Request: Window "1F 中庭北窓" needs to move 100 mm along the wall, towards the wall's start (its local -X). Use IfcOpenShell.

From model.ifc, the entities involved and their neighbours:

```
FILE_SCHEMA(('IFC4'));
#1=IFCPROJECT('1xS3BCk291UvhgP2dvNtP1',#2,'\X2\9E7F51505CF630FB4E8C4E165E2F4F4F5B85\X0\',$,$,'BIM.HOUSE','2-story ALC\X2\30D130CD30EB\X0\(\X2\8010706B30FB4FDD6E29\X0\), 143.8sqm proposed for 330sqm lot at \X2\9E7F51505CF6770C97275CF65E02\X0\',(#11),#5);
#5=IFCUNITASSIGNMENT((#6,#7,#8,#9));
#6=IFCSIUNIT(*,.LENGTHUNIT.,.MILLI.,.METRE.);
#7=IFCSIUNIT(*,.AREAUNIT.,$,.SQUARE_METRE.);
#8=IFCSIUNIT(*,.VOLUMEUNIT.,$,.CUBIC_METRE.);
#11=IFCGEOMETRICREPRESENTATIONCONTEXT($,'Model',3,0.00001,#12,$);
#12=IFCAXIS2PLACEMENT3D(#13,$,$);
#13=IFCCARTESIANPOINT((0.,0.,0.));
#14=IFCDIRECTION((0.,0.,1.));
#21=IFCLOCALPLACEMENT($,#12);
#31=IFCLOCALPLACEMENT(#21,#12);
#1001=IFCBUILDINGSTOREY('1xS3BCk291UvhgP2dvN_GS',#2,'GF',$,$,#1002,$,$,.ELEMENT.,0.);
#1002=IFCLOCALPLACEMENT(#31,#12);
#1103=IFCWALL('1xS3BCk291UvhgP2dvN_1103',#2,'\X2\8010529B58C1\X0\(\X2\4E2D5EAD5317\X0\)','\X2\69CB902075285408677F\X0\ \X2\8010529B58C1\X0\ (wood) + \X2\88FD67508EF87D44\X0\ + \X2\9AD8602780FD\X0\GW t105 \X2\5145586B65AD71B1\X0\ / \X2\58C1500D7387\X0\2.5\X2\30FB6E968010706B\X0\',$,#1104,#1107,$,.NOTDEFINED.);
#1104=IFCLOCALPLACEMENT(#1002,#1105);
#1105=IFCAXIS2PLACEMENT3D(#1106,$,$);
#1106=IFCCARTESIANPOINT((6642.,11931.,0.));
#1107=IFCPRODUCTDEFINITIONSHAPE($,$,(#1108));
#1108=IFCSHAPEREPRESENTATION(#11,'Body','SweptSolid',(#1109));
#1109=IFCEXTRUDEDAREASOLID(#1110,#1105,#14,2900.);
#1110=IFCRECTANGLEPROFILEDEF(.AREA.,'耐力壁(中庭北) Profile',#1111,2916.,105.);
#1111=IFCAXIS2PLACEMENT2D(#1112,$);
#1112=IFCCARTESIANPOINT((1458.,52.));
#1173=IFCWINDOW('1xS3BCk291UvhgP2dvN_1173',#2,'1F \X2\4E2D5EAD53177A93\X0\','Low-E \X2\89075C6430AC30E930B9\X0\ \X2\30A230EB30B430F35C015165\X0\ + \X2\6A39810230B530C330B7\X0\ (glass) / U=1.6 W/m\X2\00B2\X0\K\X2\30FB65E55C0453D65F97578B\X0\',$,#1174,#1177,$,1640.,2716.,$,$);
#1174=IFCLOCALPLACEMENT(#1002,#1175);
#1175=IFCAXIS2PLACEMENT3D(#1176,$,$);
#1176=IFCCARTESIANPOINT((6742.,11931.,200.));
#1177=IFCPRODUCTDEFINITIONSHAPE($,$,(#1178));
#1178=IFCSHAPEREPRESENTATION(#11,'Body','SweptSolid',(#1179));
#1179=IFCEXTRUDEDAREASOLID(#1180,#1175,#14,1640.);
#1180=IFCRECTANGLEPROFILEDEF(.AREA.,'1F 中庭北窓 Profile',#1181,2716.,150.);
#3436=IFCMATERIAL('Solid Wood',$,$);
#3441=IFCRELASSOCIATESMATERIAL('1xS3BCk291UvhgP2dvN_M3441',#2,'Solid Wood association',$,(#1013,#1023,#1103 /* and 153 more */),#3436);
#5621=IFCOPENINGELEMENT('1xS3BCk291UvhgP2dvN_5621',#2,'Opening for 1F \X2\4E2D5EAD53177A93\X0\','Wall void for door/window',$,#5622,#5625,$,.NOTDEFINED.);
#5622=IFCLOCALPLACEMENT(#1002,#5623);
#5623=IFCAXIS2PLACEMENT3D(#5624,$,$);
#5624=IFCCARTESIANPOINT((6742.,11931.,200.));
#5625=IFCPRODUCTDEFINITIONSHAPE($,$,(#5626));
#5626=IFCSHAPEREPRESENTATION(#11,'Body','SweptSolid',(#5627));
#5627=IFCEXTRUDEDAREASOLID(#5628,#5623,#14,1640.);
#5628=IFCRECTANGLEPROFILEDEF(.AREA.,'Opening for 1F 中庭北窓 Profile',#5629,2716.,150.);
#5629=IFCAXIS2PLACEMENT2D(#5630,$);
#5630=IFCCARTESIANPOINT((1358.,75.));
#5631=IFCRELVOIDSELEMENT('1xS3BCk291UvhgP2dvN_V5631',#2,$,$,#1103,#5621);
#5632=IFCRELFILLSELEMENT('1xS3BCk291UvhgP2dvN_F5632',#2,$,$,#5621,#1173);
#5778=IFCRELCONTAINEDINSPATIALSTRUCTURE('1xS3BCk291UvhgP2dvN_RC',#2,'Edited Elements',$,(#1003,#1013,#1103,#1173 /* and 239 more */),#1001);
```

```python
import ifcopenshell
import ifcopenshell.api.geometry
import ifcopenshell.util.placement
import ifcopenshell.util.unit

model = ifcopenshell.open("model.ifc")
unit_scale = ifcopenshell.util.unit.calculate_unit_scale(model)

window = model.by_guid("1xS3BCk291UvhgP2dvN_1173")
opening = window.FillsVoids[0].RelatingOpeningElement
wall = opening.VoidsElements[0].RelatingBuildingElement

wall_matrix = ifcopenshell.util.placement.get_local_placement(wall.ObjectPlacement)
shift = wall_matrix[:3, 0] * -0.1 / unit_scale
before = ifcopenshell.util.placement.get_local_placement(window.ObjectPlacement)[:3, 3].copy()

# The window is not placed relative to its opening, so move both.
for product in (opening, window):
    matrix = ifcopenshell.util.placement.get_local_placement(product.ObjectPlacement)
    matrix[:3, 3] += shift
    ifcopenshell.api.geometry.edit_object_placement(model, product=product, matrix=matrix, is_si=False)

after = ifcopenshell.util.placement.get_local_placement(window.ObjectPlacement)[:3, 3]
print("window moved by", (after - before).round(3) + 0.0)

model.write("model_edited.ifc")
```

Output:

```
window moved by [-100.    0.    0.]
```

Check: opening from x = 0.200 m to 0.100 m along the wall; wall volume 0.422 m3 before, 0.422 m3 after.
